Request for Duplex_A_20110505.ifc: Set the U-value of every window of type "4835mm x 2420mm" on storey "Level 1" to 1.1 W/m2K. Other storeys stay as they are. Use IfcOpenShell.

First a look at what the model holds.

```python
import ifcopenshell
import ifcopenshell.util.element

model = ifcopenshell.open("Duplex_A_20110505.ifc")
print(model.schema)
storey = next(s for s in model.by_type("IfcBuildingStorey") if s.Name == "Level 1")
windows = [e for e in ifcopenshell.util.element.get_decomposition(storey) if e.is_a("IfcWindow")]
seen = {}
for e in windows:
    element_type = ifcopenshell.util.element.get_type(e)
    key = (element_type.Name if element_type != e and element_type else None, ifcopenshell.util.element.get_pset(e, "Pset_WindowCommon", "ThermalTransmittance"))
    seen[key] = seen.get(key, 0) + 1
for (name, value), count in sorted(seen.items(), key=str):
    print(count, "x", name, "|", value)
```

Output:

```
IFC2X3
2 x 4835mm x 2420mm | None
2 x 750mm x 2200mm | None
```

```python
import ifcopenshell
import ifcopenshell.api.pset
import ifcopenshell.util.element

model = ifcopenshell.open("Duplex_A_20110505.ifc")

storey = next(s for s in model.by_type("IfcBuildingStorey") if s.Name == "Level 1")
windows = [e for e in ifcopenshell.util.element.get_decomposition(storey) if e.is_a("IfcWindow")]

count = 0
for e in windows:
    element_type = ifcopenshell.util.element.get_type(e)
    if element_type in (None, e) or element_type.Name != "4835mm x 2420mm":
        continue
    # add_pset returns the element's existing set when there is one.
    pset = ifcopenshell.api.pset.add_pset(model, product=e, name="Pset_WindowCommon")
    ifcopenshell.api.pset.edit_pset(model, pset=pset, properties={"ThermalTransmittance": 1.1})
    count += 1

print(count, "windows updated")

model.write("Duplex_A_20110505_rev.ifc")
```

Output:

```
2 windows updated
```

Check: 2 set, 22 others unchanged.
